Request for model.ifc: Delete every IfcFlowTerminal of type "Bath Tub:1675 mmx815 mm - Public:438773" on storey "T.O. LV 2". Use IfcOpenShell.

First a look at what the model holds.

```python
import ifcopenshell
import ifcopenshell.util.element

model = ifcopenshell.open("model.ifc")
print(model.schema)
storey = next(s for s in model.by_type("IfcBuildingStorey") if s.Name == "T.O. LV 2")
terminals = [e for e in ifcopenshell.util.element.get_decomposition(storey) if e.is_a("IfcFlowTerminal")]
seen = {}
for e in terminals:
    element_type = ifcopenshell.util.element.get_type(e)
    name = element_type.Name if element_type not in (None, e) else None
    seen[name] = seen.get(name, 0) + 1
for name, count in sorted(seen.items(), key=str):
    print(count, "x", name)
```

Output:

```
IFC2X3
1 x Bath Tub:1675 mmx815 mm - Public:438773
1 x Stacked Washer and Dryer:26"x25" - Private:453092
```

```python
import ifcopenshell
import ifcopenshell.api.root
import ifcopenshell.util.element

model = ifcopenshell.open("model.ifc")

storey = next(s for s in model.by_type("IfcBuildingStorey") if s.Name == "T.O. LV 2")
terminals = [e for e in ifcopenshell.util.element.get_decomposition(storey) if e.is_a("IfcFlowTerminal")]
targets = [e for e in terminals if (t := ifcopenshell.util.element.get_type(e)) not in (None, e) and t.Name == "Bath Tub:1675 mmx815 mm - Public:438773"]

for e in targets:
    ifcopenshell.api.root.remove_product(model, product=e)
print(len(targets), "removed")

model.write("model_updated.ifc")
```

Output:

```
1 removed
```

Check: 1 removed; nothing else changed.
